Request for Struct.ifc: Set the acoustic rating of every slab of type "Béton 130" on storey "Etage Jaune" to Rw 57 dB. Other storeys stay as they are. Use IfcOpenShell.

First a look at what the model holds.

```python
import ifcopenshell
import ifcopenshell.util.element

model = ifcopenshell.open("Struct.ifc")
print(model.schema)
storey = next(s for s in model.by_type("IfcBuildingStorey") if s.Name == "Etage Jaune")
slabs = [e for e in ifcopenshell.util.element.get_decomposition(storey) if e.is_a("IfcSlab")]
seen = {}
for e in slabs:
    element_type = ifcopenshell.util.element.get_type(e)
    key = (element_type.Name if element_type != e and element_type else None, ifcopenshell.util.element.get_pset(e, "Pset_SlabCommon", "AcousticRating"))
    seen[key] = seen.get(key, 0) + 1
for (name, value), count in sorted(seen.items(), key=str):
    print(count, "x", name, "|", value)
```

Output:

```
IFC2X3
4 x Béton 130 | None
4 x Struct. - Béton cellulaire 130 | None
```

```python
import ifcopenshell
import ifcopenshell.api.pset
import ifcopenshell.util.element

model = ifcopenshell.open("Struct.ifc")

storey = next(s for s in model.by_type("IfcBuildingStorey") if s.Name == "Etage Jaune")
slabs = [e for e in ifcopenshell.util.element.get_decomposition(storey) if e.is_a("IfcSlab")]

count = 0
for e in slabs:
    element_type = ifcopenshell.util.element.get_type(e)
    if element_type in (None, e) or element_type.Name != "Béton 130":
        continue
    # add_pset returns the element's existing set when there is one.
    pset = ifcopenshell.api.pset.add_pset(model, product=e, name="Pset_SlabCommon")
    ifcopenshell.api.pset.edit_pset(model, pset=pset, properties={"AcousticRating": "Rw 57 dB"})
    count += 1

print(count, "slabs updated")

model.write("Struct_updated.ifc")
```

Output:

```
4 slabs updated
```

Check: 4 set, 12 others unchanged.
